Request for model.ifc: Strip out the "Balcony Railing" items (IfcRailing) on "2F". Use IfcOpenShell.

First a look at what the model holds.

```python
import ifcopenshell
import ifcopenshell.util.element

model = ifcopenshell.open("model.ifc")
print(model.schema)
storey = next(s for s in model.by_type("IfcBuildingStorey") if s.Name == "2F")
railings = [e for e in ifcopenshell.util.element.get_decomposition(storey) if e.is_a("IfcRailing")]
seen = {}
for e in railings:
    element_type = ifcopenshell.util.element.get_type(e)
    name = element_type.Name if element_type not in (None, e) else None
    seen[name] = seen.get(name, 0) + 1
for name, count in sorted(seen.items(), key=str):
    print(count, "x", name)
```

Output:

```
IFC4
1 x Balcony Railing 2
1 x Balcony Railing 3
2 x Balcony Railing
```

```python
import ifcopenshell
import ifcopenshell.api.root
import ifcopenshell.util.element

model = ifcopenshell.open("model.ifc")

storey = next(s for s in model.by_type("IfcBuildingStorey") if s.Name == "2F")
railings = [e for e in ifcopenshell.util.element.get_decomposition(storey) if e.is_a("IfcRailing")]
targets = [e for e in railings if (t := ifcopenshell.util.element.get_type(e)) not in (None, e) and t.Name == "Balcony Railing"]

for e in targets:
    ifcopenshell.api.root.remove_product(model, product=e)
print(len(targets), "removed")

model.write("model-out.ifc")
```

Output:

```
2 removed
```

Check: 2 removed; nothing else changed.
